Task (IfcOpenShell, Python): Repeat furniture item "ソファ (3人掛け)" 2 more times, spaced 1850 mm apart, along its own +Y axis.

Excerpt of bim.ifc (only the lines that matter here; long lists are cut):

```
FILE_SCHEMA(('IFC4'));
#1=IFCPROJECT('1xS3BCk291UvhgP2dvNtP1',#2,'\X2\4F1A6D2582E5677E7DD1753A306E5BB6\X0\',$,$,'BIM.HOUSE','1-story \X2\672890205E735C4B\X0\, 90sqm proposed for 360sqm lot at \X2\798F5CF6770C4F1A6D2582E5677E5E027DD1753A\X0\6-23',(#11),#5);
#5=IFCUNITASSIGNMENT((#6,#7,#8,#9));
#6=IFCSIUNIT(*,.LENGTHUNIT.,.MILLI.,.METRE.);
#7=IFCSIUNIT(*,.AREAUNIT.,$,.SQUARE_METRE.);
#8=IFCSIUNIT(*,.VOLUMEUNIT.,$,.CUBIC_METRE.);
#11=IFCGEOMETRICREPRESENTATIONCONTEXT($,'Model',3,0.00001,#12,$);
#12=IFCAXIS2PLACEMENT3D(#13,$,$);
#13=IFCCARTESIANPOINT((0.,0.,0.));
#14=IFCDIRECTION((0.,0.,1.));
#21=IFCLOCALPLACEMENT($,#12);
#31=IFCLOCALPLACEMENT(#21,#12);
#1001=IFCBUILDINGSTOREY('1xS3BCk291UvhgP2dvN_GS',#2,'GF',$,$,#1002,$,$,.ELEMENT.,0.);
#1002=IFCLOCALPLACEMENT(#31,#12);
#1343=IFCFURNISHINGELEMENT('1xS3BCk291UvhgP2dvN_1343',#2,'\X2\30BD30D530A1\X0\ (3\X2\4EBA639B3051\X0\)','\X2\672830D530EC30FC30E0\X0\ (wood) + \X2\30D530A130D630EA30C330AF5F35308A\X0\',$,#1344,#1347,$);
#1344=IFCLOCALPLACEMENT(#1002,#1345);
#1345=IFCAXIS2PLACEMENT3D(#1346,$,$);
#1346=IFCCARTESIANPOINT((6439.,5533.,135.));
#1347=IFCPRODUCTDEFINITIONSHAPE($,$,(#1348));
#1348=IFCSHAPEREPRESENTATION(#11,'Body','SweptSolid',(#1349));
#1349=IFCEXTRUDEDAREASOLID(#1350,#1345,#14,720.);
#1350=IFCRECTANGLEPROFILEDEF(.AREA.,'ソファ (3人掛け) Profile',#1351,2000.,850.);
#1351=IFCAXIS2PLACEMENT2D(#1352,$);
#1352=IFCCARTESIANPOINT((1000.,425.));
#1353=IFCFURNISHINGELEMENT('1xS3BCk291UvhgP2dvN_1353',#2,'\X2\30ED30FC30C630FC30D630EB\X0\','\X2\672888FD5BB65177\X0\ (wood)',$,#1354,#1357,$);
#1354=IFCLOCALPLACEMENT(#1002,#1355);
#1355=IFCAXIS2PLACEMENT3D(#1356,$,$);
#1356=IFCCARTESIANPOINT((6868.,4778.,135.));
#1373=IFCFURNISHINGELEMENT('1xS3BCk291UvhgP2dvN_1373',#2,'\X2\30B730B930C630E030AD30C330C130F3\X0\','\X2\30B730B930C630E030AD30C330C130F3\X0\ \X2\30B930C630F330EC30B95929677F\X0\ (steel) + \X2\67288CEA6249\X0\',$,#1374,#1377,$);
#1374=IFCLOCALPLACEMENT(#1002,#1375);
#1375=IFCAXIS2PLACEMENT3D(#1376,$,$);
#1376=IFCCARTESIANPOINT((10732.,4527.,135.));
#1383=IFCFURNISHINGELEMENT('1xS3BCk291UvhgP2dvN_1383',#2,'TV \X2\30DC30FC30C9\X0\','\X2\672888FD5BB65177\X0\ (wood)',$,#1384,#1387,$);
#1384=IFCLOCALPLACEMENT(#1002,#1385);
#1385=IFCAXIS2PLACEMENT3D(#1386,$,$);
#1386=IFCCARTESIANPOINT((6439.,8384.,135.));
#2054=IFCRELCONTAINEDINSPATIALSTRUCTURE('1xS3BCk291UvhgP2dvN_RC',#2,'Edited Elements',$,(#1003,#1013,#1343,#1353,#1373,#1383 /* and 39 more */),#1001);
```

```python
import ifcopenshell
import ifcopenshell.api.geometry
import ifcopenshell.api.root
import ifcopenshell.util.element
import ifcopenshell.util.placement
import ifcopenshell.util.unit

model = ifcopenshell.open("bim.ifc")
unit_scale = ifcopenshell.util.unit.calculate_unit_scale(model)


def reuse_history(source, copy):
    """copy_class also copies each property set's owner history, people and application; keep the originals."""
    for rel in copy.IsDefinedBy:
        if rel.is_a("IfcRelDefinesByProperties") and (history := rel.RelatingPropertyDefinition.OwnerHistory):
            rel.RelatingPropertyDefinition.OwnerHistory = source.OwnerHistory
            ifcopenshell.util.element.remove_deep2(model, history)


source = model.by_id(1343)
base = ifcopenshell.util.placement.get_local_placement(source.ObjectPlacement)
step = base[:3, 1] * 1.85 / unit_scale

for i in range(1, 3):
    copy = ifcopenshell.api.root.copy_class(model, product=source)
    copy.Representation = ifcopenshell.util.element.copy_deep(
        model, source.Representation, exclude=["IfcGeometricRepresentationContext", "IfcRepresentationMap"]
    )
    reuse_history(source, copy)
    matrix = base.copy()
    matrix[:3, 3] += i * step
    print("added at", matrix[:3, 3].round(3) + 0.0)
    ifcopenshell.api.geometry.edit_object_placement(model, product=copy, matrix=matrix, is_si=False)

model.write("bim_v2.ifc")
```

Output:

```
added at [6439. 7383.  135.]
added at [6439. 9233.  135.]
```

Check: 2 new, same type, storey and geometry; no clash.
